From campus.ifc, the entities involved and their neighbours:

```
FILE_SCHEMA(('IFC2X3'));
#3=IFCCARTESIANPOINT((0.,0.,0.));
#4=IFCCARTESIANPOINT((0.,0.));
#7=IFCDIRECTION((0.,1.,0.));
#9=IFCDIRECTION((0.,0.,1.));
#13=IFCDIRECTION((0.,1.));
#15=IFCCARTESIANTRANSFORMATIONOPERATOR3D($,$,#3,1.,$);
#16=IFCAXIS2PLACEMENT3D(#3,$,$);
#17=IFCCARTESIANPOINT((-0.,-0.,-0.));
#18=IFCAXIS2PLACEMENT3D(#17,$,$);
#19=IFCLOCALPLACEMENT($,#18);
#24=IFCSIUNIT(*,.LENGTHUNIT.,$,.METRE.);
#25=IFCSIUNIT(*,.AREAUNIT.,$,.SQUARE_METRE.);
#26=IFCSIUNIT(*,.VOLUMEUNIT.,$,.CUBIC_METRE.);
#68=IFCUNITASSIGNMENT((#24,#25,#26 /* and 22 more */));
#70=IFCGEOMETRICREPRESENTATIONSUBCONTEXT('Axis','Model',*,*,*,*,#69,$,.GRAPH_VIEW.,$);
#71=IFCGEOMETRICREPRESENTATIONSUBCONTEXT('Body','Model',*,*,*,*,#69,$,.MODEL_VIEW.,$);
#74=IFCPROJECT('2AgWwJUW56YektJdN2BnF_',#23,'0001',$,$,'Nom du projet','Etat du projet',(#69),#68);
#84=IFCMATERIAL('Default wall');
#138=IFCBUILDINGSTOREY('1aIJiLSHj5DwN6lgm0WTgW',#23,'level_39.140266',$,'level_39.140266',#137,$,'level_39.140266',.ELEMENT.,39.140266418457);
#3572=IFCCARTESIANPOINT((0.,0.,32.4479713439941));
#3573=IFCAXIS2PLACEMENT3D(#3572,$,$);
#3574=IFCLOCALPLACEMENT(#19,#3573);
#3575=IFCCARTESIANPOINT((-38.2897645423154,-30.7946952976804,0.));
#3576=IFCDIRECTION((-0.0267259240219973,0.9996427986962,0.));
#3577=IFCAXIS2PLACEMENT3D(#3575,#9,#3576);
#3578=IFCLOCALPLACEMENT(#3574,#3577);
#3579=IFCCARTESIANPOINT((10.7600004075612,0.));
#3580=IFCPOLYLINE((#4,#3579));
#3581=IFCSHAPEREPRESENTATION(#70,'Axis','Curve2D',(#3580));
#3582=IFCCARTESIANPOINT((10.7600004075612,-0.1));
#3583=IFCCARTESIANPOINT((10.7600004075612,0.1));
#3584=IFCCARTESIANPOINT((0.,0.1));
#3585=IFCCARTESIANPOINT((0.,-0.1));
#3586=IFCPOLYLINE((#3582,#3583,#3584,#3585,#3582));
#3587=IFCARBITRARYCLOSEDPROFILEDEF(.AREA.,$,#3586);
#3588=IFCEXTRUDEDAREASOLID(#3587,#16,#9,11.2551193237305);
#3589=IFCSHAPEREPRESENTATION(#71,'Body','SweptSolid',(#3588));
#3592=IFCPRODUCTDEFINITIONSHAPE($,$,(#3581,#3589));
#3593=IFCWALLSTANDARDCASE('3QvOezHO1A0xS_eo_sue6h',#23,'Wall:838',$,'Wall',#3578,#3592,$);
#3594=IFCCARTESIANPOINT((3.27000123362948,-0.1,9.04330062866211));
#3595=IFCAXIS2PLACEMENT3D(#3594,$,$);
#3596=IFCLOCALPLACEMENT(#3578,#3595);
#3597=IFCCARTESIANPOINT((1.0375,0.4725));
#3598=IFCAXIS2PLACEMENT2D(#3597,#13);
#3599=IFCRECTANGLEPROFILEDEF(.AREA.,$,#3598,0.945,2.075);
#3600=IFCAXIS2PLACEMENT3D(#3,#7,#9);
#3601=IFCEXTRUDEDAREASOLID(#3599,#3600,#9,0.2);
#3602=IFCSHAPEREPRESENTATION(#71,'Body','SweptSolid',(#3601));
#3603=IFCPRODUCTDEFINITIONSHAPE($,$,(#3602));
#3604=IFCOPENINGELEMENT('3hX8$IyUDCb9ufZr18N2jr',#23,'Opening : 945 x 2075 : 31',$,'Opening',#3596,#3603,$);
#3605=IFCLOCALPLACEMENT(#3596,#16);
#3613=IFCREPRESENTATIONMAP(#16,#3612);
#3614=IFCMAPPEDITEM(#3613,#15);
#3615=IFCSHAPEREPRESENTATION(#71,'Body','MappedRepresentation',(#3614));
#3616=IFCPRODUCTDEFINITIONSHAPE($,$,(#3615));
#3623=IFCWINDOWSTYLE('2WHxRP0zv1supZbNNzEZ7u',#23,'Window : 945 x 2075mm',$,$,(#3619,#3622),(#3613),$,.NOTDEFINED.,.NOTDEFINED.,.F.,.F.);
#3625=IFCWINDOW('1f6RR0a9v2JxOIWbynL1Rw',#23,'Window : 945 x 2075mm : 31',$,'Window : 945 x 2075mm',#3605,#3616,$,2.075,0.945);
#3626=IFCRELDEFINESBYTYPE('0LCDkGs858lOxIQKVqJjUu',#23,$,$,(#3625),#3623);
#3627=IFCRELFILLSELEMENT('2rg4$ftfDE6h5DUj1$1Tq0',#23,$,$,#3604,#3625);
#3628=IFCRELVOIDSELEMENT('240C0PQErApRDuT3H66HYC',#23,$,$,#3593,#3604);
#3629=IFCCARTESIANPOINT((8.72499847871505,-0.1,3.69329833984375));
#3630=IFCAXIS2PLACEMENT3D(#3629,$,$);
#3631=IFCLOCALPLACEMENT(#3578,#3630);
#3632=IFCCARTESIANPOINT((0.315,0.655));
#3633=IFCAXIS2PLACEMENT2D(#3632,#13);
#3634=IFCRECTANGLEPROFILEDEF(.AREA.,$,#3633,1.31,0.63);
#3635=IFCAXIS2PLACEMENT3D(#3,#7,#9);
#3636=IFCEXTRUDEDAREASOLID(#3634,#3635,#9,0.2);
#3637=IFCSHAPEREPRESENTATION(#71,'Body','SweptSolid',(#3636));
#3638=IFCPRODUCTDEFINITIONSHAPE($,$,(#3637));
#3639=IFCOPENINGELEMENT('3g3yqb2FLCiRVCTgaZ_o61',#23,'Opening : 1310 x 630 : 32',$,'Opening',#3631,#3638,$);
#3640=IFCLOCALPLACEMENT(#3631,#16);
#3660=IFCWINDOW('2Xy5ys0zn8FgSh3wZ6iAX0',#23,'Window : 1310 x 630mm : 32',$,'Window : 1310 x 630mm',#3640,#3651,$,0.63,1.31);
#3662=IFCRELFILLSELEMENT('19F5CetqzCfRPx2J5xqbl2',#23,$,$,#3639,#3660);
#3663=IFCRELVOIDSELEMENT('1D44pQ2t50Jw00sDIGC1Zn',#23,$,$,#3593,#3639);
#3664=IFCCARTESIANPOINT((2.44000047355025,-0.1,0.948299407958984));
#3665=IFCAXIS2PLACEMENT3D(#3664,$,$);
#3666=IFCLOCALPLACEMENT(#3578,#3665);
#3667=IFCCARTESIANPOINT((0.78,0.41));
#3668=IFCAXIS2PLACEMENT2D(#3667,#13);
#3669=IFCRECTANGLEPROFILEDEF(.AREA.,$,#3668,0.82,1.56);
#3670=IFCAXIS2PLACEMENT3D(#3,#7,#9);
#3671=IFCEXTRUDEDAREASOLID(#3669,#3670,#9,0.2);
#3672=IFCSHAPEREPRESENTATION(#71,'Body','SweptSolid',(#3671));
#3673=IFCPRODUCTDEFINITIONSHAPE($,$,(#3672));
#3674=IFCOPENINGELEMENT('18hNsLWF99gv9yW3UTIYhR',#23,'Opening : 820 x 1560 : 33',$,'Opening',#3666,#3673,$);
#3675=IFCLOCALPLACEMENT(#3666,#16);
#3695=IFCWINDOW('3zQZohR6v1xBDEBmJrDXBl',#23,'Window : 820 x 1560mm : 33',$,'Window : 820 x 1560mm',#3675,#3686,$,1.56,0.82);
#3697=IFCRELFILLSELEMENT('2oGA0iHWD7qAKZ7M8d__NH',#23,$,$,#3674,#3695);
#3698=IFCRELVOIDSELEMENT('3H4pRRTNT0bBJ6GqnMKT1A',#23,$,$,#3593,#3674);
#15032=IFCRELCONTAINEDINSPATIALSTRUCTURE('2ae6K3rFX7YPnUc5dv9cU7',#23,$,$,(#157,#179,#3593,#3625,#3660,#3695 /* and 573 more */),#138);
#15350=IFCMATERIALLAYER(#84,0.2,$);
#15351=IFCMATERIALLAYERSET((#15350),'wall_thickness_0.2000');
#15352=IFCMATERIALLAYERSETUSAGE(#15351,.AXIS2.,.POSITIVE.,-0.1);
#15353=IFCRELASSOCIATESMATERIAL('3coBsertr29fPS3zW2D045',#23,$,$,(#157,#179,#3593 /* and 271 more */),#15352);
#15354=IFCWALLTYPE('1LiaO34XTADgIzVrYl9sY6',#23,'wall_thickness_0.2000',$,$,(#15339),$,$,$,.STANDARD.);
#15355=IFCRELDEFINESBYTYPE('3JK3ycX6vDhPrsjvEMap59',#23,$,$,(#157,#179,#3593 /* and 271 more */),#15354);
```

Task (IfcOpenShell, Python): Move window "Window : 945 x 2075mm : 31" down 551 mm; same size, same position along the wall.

```python
import numpy as np
import ifcopenshell
import ifcopenshell.api.geometry
import ifcopenshell.util.placement
import ifcopenshell.util.unit

model = ifcopenshell.open("campus.ifc")
unit_scale = ifcopenshell.util.unit.calculate_unit_scale(model)

window = model.by_guid("1f6RR0a9v2JxOIWbynL1Rw")
opening = window.FillsVoids[0].RelatingOpeningElement
dz = -0.551

shift = np.array([0.0, 0.0, dz])
# The window is placed relative to its opening, so it follows when the opening moves.
matrix = ifcopenshell.util.placement.get_local_placement(opening.ObjectPlacement)
matrix[:3, 3] += shift
ifcopenshell.api.geometry.edit_object_placement(
    model, product=opening, matrix=matrix, is_si=False, should_transform_children=True
)

print(f"moved by {dz * unit_scale:+.3f} m")

model.write("campus_v2.ifc")
```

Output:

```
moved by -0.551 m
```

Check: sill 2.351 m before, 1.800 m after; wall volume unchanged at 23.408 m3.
